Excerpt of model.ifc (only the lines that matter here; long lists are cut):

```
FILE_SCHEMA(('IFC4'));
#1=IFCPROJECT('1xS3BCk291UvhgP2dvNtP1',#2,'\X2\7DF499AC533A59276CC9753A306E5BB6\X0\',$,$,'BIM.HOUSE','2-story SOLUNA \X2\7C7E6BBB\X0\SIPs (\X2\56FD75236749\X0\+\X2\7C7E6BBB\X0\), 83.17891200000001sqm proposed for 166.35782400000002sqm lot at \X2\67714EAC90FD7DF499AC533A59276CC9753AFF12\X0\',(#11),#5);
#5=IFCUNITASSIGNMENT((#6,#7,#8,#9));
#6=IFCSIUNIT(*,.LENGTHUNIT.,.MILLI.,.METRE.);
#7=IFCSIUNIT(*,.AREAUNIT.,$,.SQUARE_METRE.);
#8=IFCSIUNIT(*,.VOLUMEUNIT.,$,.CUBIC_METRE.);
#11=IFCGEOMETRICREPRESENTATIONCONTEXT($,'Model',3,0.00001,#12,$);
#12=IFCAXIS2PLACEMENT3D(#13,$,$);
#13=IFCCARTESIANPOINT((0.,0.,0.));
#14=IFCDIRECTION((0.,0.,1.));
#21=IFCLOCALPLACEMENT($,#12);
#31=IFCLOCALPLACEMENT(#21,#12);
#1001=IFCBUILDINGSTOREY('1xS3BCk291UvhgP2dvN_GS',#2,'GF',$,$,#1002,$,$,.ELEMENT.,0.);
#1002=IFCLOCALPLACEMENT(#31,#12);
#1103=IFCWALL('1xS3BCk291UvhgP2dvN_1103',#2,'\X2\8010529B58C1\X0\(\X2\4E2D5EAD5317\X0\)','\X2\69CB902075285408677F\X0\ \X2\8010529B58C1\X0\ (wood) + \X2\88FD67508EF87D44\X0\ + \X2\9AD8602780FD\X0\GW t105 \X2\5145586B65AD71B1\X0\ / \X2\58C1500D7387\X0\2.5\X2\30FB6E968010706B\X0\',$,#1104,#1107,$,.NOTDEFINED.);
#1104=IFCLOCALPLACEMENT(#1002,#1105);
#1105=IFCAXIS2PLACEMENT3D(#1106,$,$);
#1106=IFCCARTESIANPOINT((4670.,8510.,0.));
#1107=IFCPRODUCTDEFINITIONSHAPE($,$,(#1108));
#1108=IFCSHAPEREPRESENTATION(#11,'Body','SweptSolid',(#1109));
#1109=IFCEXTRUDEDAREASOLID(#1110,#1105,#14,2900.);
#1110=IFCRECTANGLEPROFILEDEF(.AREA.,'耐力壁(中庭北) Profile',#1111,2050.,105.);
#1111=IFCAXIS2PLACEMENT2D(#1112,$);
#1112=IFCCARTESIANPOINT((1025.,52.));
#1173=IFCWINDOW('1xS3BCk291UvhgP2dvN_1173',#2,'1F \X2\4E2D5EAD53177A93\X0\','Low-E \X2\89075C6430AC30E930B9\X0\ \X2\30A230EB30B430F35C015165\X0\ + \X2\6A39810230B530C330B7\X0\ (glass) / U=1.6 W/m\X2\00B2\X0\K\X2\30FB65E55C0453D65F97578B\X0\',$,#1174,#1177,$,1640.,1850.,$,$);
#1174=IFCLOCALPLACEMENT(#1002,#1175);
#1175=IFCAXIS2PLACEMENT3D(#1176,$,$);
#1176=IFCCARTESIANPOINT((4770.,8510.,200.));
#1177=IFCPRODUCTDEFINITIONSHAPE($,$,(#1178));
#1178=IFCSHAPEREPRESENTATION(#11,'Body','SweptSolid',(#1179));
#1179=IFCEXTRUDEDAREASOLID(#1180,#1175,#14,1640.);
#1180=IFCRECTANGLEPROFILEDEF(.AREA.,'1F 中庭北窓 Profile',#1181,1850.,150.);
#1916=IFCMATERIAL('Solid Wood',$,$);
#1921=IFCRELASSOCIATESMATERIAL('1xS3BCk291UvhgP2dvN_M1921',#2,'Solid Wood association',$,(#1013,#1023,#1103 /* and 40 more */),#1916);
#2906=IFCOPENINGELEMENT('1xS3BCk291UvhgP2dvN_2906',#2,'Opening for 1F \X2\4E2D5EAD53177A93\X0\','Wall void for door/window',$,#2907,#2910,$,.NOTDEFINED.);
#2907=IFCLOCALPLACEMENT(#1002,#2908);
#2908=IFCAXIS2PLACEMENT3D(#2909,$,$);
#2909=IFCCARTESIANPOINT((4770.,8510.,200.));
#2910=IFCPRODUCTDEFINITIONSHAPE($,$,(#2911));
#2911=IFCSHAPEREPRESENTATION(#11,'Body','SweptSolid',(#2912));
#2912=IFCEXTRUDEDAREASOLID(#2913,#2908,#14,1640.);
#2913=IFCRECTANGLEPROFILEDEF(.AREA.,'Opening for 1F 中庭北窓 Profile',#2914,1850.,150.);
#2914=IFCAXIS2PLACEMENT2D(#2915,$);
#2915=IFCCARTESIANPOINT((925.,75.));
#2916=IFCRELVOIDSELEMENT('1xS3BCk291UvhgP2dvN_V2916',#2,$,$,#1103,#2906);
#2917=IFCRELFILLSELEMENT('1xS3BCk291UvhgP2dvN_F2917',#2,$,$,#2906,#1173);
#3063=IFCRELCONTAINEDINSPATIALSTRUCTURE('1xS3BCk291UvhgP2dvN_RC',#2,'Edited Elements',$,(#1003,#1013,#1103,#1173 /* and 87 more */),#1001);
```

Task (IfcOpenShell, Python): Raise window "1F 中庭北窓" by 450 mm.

```python
import numpy as np
import ifcopenshell
import ifcopenshell.api.geometry
import ifcopenshell.util.placement
import ifcopenshell.util.unit

model = ifcopenshell.open("model.ifc")
unit_scale = ifcopenshell.util.unit.calculate_unit_scale(model)

window = model.by_guid("1xS3BCk291UvhgP2dvN_1173")
opening = window.FillsVoids[0].RelatingOpeningElement
dz = 450.0

shift = np.array([0.0, 0.0, dz])
# The window is not placed relative to its opening, so move both.
for product in (opening, window):
    matrix = ifcopenshell.util.placement.get_local_placement(product.ObjectPlacement)
    matrix[:3, 3] += shift
    ifcopenshell.api.geometry.edit_object_placement(model, product=product, matrix=matrix, is_si=False)

print(f"moved by {dz * unit_scale:+.3f} m")

model.write("model_rev.ifc")
```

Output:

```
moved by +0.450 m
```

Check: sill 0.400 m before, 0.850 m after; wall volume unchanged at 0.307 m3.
